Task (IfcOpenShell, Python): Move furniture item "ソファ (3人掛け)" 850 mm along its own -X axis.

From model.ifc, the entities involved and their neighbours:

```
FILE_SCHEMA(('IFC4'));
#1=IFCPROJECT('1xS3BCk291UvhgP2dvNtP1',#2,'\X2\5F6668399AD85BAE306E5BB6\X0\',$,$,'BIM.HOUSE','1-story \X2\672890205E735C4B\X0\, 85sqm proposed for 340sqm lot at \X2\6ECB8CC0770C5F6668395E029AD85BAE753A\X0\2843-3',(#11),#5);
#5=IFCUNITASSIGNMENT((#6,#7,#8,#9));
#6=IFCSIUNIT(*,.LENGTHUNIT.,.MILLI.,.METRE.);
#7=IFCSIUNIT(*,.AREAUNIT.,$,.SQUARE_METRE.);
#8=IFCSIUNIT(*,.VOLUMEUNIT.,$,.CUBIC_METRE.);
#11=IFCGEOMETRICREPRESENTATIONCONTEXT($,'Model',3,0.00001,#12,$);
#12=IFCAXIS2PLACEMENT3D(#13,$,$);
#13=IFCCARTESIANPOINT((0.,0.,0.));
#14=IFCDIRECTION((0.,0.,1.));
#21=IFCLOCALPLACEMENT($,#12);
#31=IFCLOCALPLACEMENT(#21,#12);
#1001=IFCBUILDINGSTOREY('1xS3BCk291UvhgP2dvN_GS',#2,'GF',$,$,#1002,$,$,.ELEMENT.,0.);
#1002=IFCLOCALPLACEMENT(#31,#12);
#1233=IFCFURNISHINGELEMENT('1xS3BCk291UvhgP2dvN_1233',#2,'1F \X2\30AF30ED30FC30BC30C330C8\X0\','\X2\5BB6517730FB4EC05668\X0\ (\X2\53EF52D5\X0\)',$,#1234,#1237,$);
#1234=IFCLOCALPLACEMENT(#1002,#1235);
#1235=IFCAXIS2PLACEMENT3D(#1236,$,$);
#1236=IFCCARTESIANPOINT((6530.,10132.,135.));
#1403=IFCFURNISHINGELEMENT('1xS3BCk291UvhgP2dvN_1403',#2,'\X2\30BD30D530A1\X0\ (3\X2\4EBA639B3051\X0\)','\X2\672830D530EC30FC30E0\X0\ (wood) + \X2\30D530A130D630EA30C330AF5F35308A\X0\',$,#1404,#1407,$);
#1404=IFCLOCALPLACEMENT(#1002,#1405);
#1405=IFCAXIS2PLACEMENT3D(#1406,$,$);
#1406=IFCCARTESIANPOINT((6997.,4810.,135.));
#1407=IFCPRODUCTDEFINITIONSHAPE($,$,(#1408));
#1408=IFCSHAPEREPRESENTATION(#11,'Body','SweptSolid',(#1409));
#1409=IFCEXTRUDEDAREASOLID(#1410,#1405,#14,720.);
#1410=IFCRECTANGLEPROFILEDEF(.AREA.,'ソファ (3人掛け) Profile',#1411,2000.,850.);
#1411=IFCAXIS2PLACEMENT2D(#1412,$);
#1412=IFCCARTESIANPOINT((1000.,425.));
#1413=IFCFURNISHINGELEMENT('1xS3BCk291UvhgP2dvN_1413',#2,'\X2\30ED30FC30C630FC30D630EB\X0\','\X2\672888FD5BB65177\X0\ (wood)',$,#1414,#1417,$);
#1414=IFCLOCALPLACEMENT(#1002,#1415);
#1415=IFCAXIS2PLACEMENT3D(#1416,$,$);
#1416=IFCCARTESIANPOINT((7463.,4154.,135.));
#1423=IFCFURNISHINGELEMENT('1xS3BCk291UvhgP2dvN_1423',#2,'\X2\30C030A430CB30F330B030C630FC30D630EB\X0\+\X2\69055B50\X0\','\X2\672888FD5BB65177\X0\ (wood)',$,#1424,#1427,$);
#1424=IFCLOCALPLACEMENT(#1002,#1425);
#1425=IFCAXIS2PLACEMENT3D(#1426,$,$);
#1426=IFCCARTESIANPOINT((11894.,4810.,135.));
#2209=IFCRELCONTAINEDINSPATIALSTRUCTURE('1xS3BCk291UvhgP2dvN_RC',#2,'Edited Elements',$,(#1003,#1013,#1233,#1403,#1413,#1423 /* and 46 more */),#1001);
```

```python
import ifcopenshell
import ifcopenshell.api.geometry
import ifcopenshell.util.placement

model = ifcopenshell.open("model.ifc")

item = model.by_id(1403)
matrix = ifcopenshell.util.placement.get_local_placement(item.ObjectPlacement)
matrix[:3, 3] -= matrix[:3, 0] * 850.0
ifcopenshell.api.geometry.edit_object_placement(model, product=item, matrix=matrix, is_si=False)

print(ifcopenshell.util.placement.get_local_placement(item.ObjectPlacement).round(3) + 0.0)

model.write("model_v2.ifc")
```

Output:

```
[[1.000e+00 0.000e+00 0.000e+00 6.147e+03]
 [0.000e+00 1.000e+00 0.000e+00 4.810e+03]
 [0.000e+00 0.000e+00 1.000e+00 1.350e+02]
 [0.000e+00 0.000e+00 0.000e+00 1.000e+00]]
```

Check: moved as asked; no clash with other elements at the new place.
